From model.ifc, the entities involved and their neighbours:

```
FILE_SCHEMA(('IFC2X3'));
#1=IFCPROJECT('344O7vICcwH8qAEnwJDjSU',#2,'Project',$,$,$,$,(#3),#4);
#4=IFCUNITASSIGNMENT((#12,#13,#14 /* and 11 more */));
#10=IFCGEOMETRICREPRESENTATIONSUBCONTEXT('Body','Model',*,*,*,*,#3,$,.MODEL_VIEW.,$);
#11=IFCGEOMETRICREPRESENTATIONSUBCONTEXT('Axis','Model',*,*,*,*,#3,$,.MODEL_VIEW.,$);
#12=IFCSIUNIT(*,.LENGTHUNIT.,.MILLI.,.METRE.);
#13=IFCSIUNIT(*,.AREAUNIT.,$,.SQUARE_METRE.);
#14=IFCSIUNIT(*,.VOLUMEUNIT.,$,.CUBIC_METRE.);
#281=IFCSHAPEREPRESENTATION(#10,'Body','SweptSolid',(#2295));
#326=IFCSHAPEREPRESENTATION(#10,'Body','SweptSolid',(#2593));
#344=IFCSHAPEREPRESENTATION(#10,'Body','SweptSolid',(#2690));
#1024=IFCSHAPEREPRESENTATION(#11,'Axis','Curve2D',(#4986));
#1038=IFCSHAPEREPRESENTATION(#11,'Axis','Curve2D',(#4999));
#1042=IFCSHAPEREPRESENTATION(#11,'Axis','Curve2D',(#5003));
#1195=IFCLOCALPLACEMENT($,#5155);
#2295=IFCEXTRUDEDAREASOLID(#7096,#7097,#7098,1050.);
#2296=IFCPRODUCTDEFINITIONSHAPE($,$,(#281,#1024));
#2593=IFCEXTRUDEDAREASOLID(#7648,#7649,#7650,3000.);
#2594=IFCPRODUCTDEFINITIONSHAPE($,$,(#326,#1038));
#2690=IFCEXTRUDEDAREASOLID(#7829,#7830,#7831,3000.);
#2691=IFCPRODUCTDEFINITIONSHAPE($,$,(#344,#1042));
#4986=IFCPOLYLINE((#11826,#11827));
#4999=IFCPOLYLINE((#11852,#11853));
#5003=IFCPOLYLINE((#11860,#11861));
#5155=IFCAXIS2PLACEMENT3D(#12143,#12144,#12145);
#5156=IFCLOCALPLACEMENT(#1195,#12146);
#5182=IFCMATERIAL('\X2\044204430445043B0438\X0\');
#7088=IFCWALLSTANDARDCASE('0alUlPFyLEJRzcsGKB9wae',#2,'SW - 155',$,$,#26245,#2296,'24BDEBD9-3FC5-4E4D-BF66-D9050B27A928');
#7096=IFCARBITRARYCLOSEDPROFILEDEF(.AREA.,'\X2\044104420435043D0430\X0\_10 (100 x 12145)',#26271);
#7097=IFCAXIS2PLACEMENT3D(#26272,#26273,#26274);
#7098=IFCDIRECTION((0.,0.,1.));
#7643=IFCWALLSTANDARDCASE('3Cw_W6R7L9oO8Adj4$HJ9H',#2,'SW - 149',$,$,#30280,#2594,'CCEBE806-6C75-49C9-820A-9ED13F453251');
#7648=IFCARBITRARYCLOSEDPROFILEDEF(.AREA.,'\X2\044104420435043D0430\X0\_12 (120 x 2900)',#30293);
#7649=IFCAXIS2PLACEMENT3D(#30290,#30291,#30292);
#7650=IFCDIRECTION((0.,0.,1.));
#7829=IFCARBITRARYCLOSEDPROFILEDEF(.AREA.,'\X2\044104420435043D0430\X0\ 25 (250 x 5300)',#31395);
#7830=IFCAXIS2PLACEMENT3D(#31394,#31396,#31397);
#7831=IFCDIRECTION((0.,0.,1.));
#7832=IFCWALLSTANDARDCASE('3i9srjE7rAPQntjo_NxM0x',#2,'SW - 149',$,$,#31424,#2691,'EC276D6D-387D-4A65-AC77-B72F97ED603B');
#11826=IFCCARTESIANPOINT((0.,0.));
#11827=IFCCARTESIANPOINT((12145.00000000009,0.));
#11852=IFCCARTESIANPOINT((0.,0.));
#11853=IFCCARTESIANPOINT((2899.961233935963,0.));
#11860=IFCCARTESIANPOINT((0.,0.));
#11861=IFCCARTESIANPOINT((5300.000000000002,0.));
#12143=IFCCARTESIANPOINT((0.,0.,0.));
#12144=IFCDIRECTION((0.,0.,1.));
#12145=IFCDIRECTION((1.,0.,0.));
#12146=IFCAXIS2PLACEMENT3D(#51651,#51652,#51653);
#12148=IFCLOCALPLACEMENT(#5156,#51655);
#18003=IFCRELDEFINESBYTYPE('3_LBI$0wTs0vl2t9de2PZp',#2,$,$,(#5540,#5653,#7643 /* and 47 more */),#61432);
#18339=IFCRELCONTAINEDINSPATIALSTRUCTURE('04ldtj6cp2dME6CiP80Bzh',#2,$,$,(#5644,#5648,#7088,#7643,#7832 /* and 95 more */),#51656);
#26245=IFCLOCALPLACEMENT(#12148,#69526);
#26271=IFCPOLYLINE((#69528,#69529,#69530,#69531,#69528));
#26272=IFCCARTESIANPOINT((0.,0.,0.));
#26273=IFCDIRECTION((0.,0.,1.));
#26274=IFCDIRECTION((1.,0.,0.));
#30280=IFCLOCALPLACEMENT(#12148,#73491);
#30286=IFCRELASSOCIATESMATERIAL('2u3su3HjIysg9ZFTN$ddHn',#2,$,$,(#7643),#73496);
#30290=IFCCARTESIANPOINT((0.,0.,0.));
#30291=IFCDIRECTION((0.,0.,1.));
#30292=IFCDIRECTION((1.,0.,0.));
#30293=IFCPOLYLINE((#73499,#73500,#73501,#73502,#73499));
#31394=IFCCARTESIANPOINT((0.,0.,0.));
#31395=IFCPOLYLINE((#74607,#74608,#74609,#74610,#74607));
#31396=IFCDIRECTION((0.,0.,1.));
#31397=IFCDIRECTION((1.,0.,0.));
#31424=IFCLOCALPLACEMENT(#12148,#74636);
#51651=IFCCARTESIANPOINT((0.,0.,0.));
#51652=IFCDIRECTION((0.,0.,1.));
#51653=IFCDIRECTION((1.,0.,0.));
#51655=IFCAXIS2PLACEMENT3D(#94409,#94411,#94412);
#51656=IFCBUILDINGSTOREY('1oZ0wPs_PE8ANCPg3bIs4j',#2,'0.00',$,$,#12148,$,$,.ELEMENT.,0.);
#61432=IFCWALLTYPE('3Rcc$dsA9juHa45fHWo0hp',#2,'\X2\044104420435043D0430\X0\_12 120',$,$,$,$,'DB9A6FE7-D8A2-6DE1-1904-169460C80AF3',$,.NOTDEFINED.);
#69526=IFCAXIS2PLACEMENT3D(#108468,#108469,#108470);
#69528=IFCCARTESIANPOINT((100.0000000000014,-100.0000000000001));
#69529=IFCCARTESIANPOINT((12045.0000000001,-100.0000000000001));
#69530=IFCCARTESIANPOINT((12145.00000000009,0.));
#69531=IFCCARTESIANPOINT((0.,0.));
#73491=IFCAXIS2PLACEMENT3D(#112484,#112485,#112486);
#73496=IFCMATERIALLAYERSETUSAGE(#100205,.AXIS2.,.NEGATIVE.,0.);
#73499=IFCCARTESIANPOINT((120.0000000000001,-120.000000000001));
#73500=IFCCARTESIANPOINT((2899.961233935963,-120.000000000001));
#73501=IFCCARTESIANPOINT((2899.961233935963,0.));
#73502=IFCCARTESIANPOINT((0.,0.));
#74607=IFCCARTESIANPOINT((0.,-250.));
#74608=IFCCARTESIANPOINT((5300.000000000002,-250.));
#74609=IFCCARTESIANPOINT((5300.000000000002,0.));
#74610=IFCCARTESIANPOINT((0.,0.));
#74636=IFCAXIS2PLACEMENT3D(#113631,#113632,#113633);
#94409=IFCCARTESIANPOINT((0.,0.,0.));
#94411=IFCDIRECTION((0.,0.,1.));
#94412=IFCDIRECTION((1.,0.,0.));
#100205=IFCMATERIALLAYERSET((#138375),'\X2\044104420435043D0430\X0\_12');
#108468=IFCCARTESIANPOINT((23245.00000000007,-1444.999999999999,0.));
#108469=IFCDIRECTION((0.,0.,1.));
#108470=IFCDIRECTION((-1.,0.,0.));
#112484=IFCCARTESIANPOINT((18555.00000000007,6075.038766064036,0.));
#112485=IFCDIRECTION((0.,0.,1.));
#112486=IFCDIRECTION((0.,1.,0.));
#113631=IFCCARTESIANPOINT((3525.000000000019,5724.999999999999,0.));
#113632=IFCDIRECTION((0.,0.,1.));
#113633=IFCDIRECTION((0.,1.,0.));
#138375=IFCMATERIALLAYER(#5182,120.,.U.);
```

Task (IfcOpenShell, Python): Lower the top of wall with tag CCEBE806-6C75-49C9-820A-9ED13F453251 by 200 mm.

```python
import ifcopenshell
import ifcopenshell.geom
import ifcopenshell.util.representation
import ifcopenshell.util.shape
import ifcopenshell.util.unit

model = ifcopenshell.open("model.ifc")
unit_scale = ifcopenshell.util.unit.calculate_unit_scale(model)
settings = ifcopenshell.geom.settings()


def volume(element):
    """Net volume in cubic metres, openings subtracted."""
    shape = ifcopenshell.geom.create_shape(settings, element)
    return ifcopenshell.util.shape.get_volume(shape.geometry)


wall = model.by_guid("3Cw_W6R7L9oO8Adj4$HJ9H")
before = volume(wall)

body = ifcopenshell.util.representation.get_representation(wall, "Model", "Body")
solid = body.Items[0]
old_height = solid.Depth
solid.Depth -= 0.2 / unit_scale
after = volume(wall)

print(f"height {old_height:g} -> {solid.Depth:g}, volume {before:.3f} -> {after:.3f} m3")

model.write("model_edited.ifc")
```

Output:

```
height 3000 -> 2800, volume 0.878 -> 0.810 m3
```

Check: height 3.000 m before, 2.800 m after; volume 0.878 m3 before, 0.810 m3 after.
